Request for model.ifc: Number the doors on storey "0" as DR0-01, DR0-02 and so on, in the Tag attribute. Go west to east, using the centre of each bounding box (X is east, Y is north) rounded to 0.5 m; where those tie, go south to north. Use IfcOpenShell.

First a look at what the model holds.

```python
import ifcopenshell
import ifcopenshell.util.element
import ifcopenshell.util.placement

model = ifcopenshell.open("model.ifc")
print(model.schema)
storey = next(s for s in model.by_type("IfcBuildingStorey") if s.Name == "0")
doors = [e for e in ifcopenshell.util.element.get_decomposition(storey) if e.is_a("IfcDoor")]
for e in sorted(doors, key=lambda e: e.id()):
    origin = ifcopenshell.util.placement.get_local_placement(e.ObjectPlacement)[:3, 3]
    print(e.id(), e.Tag, e.Name, origin.round(2) + 0.0, sep=" | ")
```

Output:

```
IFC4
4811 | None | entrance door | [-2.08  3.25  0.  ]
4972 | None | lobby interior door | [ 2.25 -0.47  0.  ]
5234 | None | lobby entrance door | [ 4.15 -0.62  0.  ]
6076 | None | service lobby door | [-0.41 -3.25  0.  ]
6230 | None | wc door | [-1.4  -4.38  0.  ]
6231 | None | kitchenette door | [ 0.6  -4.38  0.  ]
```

```python
import ifcopenshell
import ifcopenshell.geom
import ifcopenshell.util.element
import ifcopenshell.util.shape

model = ifcopenshell.open("model.ifc")
settings = ifcopenshell.geom.settings()
settings.set("use-world-coords", True)


def centre(element):
    shape = ifcopenshell.geom.create_shape(settings, element)
    return ifcopenshell.util.shape.get_bbox_centroid(shape.geometry)


storey = next(s for s in model.by_type("IfcBuildingStorey") if s.Name == "0")
doors = [e for e in ifcopenshell.util.element.get_decomposition(storey) if e.is_a("IfcDoor")]

# Insertion points can sit at a corner or the storey origin, so sort by the geometry (in metres).
centres = {e: centre(e) for e in doors}
doors.sort(key=lambda e: (round(centres[e][0] / 0.5), centres[e][1]))

for i, e in enumerate(doors, start=1):
    number = f"DR0-{i:02d}"
    e.Tag = number
    print(e.id(), number)

model.write("model_v2.ifc")
```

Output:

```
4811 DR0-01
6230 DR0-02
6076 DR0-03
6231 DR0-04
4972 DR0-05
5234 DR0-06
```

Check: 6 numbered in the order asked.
